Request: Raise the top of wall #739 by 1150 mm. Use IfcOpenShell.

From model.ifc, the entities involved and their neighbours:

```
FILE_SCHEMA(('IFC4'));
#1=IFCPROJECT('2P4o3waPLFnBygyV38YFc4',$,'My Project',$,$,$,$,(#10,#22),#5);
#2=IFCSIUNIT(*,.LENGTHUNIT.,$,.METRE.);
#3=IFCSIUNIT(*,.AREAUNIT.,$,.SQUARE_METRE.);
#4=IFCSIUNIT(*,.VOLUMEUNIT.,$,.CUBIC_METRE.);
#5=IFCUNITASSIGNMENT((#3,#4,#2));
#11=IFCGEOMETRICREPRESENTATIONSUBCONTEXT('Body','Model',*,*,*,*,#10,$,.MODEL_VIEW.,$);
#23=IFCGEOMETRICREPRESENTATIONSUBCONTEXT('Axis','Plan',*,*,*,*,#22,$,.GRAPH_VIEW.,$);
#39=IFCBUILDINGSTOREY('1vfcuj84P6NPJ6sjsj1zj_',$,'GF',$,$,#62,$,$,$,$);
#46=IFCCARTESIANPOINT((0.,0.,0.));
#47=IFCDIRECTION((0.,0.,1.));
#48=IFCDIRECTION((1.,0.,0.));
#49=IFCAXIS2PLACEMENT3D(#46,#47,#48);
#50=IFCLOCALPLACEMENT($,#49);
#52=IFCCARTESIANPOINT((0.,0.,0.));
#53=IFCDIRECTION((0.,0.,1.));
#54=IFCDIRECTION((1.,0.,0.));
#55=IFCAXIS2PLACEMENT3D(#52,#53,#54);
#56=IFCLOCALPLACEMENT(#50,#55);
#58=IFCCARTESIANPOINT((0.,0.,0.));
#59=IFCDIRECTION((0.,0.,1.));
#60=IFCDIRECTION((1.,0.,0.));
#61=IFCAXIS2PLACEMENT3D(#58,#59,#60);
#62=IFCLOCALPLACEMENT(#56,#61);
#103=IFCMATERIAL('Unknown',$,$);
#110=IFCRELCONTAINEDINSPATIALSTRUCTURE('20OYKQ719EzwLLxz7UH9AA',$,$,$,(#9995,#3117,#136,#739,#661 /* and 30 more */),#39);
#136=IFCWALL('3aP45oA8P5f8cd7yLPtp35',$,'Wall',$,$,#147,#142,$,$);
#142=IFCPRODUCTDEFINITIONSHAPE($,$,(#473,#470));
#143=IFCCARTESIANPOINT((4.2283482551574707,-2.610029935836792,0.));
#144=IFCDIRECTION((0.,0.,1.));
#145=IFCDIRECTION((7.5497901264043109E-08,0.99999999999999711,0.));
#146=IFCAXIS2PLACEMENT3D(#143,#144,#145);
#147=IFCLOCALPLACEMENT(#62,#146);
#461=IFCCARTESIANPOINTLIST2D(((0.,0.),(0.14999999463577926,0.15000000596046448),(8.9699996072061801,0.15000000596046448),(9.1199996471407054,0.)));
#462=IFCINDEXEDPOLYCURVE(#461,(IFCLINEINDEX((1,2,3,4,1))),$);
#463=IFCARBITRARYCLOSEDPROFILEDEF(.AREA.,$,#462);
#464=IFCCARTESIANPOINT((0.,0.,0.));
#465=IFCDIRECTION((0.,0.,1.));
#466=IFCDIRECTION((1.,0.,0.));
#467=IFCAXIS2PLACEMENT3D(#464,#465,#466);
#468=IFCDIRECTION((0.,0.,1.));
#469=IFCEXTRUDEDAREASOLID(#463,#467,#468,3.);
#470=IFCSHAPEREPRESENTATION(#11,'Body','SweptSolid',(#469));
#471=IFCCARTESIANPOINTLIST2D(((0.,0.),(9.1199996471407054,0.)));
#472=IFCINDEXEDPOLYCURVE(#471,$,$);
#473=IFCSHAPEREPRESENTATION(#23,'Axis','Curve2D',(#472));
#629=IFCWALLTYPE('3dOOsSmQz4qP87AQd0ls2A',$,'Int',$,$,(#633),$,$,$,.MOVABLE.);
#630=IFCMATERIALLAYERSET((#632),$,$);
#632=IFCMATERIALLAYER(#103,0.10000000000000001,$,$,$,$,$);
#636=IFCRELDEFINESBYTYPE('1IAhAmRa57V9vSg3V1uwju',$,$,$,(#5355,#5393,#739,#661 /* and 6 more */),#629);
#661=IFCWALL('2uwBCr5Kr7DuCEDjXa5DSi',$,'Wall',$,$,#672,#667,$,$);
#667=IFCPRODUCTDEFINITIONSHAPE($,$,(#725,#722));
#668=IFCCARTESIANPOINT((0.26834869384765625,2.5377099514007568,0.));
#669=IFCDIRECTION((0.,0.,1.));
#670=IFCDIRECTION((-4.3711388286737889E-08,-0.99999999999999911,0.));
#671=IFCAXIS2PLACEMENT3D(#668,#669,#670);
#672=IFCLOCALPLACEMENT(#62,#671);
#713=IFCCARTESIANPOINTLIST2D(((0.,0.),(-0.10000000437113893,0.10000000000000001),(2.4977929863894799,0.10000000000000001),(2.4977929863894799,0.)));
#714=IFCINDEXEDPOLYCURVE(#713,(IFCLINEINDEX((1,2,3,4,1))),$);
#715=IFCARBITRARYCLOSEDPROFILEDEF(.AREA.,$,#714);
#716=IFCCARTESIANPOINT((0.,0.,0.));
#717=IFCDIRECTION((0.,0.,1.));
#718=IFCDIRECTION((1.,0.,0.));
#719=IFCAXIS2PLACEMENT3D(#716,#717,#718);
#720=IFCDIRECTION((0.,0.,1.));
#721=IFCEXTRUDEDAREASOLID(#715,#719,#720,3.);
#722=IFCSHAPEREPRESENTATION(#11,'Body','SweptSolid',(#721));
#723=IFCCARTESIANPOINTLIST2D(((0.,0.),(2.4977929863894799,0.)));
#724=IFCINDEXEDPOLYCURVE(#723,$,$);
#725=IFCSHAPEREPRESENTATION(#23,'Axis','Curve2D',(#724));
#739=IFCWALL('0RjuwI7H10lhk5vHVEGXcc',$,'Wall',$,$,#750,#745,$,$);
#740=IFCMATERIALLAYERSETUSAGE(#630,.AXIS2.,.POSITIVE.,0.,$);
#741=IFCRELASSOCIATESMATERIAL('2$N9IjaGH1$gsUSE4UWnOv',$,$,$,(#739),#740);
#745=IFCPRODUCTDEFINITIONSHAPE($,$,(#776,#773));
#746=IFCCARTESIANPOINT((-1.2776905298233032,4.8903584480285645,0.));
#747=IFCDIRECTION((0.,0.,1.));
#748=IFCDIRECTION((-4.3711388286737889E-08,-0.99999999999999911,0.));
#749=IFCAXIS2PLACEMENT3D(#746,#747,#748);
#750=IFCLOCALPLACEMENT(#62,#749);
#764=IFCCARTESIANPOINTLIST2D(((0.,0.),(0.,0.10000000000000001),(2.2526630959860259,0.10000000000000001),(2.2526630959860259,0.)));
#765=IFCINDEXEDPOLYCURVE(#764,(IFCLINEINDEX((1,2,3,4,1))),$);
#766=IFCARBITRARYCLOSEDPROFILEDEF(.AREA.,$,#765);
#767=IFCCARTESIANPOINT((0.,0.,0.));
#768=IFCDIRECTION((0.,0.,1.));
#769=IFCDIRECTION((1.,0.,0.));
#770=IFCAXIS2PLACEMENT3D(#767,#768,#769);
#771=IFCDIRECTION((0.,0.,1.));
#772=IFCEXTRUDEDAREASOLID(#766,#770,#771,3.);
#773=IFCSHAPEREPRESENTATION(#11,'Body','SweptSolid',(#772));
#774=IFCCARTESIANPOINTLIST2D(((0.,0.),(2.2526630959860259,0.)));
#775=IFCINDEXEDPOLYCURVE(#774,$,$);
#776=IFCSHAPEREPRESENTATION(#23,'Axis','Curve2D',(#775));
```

```python
import ifcopenshell
import ifcopenshell.geom
import ifcopenshell.util.representation
import ifcopenshell.util.shape

model = ifcopenshell.open("model.ifc")
settings = ifcopenshell.geom.settings()


def volume(element):
    """Net volume in cubic metres, openings subtracted."""
    shape = ifcopenshell.geom.create_shape(settings, element)
    return ifcopenshell.util.shape.get_volume(shape.geometry)


wall = model.by_guid("0RjuwI7H10lhk5vHVEGXcc")
before = volume(wall)

body = ifcopenshell.util.representation.get_representation(wall, "Model", "Body")
solid = body.Items[0]
old_height = solid.Depth
solid.Depth += 1.15
after = volume(wall)

print(f"height {old_height:g} -> {solid.Depth:g}, volume {before:.3f} -> {after:.3f} m3")

model.write("model_v2.ifc")
```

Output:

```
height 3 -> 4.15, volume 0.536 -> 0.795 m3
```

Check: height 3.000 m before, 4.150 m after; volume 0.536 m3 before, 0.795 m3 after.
